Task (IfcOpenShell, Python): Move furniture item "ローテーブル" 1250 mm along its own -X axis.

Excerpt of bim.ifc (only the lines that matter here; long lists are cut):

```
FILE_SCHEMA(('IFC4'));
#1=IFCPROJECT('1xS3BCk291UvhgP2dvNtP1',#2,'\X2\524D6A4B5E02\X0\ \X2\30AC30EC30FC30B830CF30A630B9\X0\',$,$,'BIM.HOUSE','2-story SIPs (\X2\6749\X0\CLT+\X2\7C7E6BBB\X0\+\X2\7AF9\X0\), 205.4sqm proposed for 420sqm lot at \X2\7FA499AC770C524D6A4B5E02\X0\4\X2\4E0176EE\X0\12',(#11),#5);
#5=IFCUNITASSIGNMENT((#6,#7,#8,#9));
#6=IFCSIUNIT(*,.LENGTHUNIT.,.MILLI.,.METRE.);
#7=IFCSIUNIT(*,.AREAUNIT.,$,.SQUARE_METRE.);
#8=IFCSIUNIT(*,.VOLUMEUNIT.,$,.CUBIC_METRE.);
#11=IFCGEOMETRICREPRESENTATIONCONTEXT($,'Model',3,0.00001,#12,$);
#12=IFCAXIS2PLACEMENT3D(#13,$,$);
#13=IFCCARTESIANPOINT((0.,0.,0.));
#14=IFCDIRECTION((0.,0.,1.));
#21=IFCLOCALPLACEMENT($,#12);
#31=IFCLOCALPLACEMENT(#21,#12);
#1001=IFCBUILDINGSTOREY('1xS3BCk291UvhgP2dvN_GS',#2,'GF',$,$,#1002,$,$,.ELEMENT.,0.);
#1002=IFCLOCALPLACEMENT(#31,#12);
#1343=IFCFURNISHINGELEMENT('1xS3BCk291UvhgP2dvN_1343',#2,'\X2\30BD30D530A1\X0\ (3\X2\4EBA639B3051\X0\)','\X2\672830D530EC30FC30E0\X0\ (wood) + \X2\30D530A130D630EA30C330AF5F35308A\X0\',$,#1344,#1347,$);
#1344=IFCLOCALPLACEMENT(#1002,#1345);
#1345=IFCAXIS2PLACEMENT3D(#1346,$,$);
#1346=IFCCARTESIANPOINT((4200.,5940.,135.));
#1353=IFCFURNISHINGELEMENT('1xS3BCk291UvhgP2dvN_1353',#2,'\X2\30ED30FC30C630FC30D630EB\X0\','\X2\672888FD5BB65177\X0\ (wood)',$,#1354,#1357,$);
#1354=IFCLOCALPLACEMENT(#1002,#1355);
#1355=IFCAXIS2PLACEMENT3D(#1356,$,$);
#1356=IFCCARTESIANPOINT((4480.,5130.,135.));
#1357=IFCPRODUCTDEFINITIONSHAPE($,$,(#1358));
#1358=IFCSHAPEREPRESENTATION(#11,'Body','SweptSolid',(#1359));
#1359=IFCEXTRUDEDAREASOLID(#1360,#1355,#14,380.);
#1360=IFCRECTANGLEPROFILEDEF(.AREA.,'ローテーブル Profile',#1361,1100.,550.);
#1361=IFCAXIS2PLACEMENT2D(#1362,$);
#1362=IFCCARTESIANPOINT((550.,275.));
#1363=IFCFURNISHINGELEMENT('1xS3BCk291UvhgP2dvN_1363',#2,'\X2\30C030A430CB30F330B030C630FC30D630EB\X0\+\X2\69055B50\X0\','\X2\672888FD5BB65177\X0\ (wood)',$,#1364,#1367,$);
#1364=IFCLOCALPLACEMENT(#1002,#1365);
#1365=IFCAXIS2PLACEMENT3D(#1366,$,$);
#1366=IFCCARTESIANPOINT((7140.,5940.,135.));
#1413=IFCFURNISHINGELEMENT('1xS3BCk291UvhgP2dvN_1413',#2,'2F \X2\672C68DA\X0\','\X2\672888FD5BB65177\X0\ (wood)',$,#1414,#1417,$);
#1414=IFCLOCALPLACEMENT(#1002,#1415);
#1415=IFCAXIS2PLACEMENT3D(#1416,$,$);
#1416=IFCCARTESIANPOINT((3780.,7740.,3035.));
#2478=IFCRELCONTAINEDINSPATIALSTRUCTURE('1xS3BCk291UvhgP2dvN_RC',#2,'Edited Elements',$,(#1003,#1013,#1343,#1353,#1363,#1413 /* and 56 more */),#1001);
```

```python
import ifcopenshell
import ifcopenshell.api.geometry
import ifcopenshell.util.placement
import ifcopenshell.util.unit

model = ifcopenshell.open("bim.ifc")
unit_scale = ifcopenshell.util.unit.calculate_unit_scale(model)

item = model.by_guid("1xS3BCk291UvhgP2dvN_1353")
matrix = ifcopenshell.util.placement.get_local_placement(item.ObjectPlacement)
matrix[:3, 3] -= matrix[:3, 0] * 1.25 / unit_scale
ifcopenshell.api.geometry.edit_object_placement(model, product=item, matrix=matrix, is_si=False)

print(ifcopenshell.util.placement.get_local_placement(item.ObjectPlacement).round(3) + 0.0)

model.write("bim-out.ifc")
```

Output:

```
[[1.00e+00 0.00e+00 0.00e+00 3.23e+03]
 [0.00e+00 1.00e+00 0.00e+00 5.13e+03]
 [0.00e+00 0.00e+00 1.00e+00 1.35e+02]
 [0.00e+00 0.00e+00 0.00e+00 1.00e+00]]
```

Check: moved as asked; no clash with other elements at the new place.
